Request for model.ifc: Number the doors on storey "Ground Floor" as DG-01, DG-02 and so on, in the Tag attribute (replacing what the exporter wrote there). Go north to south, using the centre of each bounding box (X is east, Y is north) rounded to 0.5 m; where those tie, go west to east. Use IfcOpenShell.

First a look at what the model holds.

```python
import ifcopenshell
import ifcopenshell.util.element
import ifcopenshell.util.placement

model = ifcopenshell.open("model.ifc")
print(model.schema)
storey = next(s for s in model.by_type("IfcBuildingStorey") if s.Name == "Ground Floor")
doors = [e for e in ifcopenshell.util.element.get_decomposition(storey) if e.is_a("IfcDoor")]
for e in sorted(doors, key=lambda e: e.id()):
    origin = ifcopenshell.util.placement.get_local_placement(e.ObjectPlacement)[:3, 3]
    print(e.id(), e.Tag, e.Name, origin.round(2) + 0.0, sep=" | ")
```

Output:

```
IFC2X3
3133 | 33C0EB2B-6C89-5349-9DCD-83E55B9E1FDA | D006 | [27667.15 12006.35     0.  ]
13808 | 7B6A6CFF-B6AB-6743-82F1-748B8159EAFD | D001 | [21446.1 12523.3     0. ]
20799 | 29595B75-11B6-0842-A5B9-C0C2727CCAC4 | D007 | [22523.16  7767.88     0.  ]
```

```python
import ifcopenshell
import ifcopenshell.geom
import ifcopenshell.util.element
import ifcopenshell.util.shape

model = ifcopenshell.open("model.ifc")
settings = ifcopenshell.geom.settings()
settings.set("use-world-coords", True)


def centre(element):
    shape = ifcopenshell.geom.create_shape(settings, element)
    return ifcopenshell.util.shape.get_bbox_centroid(shape.geometry)


storey = next(s for s in model.by_type("IfcBuildingStorey") if s.Name == "Ground Floor")
doors = [e for e in ifcopenshell.util.element.get_decomposition(storey) if e.is_a("IfcDoor")]

# Insertion points can sit at a corner or the storey origin, so sort by the geometry (in metres).
centres = {e: centre(e) for e in doors}
doors.sort(key=lambda e: (-round(centres[e][1] / 0.5), centres[e][0]))

for i, e in enumerate(doors, start=1):
    number = f"DG-{i:02d}"
    e.Tag = number
    print(e.id(), number)

model.write("model_rev.ifc")
```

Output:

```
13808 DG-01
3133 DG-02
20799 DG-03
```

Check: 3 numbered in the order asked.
